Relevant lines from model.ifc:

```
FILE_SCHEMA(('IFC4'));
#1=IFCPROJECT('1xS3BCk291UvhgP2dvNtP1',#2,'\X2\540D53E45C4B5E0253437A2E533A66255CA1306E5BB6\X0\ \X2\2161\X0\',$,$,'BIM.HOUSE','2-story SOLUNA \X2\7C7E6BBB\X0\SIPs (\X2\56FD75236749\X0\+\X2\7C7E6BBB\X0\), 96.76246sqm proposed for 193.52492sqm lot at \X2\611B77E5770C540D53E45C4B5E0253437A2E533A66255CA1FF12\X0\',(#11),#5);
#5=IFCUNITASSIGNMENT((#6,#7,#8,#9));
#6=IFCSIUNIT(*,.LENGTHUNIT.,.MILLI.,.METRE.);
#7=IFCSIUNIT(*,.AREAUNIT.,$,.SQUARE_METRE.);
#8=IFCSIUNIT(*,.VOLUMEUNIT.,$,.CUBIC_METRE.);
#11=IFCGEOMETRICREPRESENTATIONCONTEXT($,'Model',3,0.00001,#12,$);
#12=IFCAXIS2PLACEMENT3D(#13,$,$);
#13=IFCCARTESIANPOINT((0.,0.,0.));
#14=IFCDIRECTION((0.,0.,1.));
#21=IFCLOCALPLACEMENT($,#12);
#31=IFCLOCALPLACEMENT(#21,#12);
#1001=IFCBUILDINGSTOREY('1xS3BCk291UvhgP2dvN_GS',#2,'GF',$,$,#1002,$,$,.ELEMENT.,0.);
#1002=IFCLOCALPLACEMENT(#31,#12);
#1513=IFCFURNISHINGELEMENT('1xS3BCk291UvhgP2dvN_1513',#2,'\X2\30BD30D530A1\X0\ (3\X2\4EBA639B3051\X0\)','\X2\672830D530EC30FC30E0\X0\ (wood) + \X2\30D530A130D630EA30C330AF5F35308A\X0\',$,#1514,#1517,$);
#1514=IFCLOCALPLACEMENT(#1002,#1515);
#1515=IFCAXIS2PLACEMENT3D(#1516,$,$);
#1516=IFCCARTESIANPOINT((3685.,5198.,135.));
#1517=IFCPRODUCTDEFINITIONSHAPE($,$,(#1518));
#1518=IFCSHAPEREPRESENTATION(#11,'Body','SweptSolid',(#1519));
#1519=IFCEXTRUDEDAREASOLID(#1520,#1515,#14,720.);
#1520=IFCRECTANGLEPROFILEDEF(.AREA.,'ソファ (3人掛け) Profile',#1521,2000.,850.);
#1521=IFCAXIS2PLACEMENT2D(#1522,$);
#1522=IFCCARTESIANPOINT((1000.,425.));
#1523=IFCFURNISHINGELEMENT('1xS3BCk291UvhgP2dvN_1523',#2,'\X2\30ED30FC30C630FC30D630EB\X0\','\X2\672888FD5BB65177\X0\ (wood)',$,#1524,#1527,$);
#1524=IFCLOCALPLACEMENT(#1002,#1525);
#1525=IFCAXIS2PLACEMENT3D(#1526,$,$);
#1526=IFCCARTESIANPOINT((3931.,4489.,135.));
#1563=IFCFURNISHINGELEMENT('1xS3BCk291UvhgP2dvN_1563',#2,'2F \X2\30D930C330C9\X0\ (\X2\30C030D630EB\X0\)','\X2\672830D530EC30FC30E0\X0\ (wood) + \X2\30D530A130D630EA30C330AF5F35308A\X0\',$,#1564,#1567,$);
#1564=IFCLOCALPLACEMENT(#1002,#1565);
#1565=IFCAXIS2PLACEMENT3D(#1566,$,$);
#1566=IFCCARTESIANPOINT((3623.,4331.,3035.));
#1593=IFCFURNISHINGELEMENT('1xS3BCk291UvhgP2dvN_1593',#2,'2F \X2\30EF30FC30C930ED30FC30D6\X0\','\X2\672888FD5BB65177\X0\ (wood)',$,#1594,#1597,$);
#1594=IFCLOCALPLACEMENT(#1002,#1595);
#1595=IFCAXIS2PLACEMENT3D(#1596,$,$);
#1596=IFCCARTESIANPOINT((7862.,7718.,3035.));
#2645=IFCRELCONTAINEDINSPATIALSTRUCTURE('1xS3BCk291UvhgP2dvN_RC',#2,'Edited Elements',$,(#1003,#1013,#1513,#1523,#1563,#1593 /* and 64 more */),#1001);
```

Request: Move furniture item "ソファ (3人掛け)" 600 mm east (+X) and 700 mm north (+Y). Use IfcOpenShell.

```python
import ifcopenshell
import ifcopenshell.api.geometry
import ifcopenshell.util.placement
import ifcopenshell.util.unit

model = ifcopenshell.open("model.ifc")
unit_scale = ifcopenshell.util.unit.calculate_unit_scale(model)

item = model.by_guid("1xS3BCk291UvhgP2dvN_1513")
matrix = ifcopenshell.util.placement.get_local_placement(item.ObjectPlacement)
matrix[0, 3] += 0.6 / unit_scale
matrix[1, 3] += 0.7 / unit_scale
ifcopenshell.api.geometry.edit_object_placement(model, product=item, matrix=matrix, is_si=False)

print(ifcopenshell.util.placement.get_local_placement(item.ObjectPlacement).round(3) + 0.0)

model.write("model_updated.ifc")
```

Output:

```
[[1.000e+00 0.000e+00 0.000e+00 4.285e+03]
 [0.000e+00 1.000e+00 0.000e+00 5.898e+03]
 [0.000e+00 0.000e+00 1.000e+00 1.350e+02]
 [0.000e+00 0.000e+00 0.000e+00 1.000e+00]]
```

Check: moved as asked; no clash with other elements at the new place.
